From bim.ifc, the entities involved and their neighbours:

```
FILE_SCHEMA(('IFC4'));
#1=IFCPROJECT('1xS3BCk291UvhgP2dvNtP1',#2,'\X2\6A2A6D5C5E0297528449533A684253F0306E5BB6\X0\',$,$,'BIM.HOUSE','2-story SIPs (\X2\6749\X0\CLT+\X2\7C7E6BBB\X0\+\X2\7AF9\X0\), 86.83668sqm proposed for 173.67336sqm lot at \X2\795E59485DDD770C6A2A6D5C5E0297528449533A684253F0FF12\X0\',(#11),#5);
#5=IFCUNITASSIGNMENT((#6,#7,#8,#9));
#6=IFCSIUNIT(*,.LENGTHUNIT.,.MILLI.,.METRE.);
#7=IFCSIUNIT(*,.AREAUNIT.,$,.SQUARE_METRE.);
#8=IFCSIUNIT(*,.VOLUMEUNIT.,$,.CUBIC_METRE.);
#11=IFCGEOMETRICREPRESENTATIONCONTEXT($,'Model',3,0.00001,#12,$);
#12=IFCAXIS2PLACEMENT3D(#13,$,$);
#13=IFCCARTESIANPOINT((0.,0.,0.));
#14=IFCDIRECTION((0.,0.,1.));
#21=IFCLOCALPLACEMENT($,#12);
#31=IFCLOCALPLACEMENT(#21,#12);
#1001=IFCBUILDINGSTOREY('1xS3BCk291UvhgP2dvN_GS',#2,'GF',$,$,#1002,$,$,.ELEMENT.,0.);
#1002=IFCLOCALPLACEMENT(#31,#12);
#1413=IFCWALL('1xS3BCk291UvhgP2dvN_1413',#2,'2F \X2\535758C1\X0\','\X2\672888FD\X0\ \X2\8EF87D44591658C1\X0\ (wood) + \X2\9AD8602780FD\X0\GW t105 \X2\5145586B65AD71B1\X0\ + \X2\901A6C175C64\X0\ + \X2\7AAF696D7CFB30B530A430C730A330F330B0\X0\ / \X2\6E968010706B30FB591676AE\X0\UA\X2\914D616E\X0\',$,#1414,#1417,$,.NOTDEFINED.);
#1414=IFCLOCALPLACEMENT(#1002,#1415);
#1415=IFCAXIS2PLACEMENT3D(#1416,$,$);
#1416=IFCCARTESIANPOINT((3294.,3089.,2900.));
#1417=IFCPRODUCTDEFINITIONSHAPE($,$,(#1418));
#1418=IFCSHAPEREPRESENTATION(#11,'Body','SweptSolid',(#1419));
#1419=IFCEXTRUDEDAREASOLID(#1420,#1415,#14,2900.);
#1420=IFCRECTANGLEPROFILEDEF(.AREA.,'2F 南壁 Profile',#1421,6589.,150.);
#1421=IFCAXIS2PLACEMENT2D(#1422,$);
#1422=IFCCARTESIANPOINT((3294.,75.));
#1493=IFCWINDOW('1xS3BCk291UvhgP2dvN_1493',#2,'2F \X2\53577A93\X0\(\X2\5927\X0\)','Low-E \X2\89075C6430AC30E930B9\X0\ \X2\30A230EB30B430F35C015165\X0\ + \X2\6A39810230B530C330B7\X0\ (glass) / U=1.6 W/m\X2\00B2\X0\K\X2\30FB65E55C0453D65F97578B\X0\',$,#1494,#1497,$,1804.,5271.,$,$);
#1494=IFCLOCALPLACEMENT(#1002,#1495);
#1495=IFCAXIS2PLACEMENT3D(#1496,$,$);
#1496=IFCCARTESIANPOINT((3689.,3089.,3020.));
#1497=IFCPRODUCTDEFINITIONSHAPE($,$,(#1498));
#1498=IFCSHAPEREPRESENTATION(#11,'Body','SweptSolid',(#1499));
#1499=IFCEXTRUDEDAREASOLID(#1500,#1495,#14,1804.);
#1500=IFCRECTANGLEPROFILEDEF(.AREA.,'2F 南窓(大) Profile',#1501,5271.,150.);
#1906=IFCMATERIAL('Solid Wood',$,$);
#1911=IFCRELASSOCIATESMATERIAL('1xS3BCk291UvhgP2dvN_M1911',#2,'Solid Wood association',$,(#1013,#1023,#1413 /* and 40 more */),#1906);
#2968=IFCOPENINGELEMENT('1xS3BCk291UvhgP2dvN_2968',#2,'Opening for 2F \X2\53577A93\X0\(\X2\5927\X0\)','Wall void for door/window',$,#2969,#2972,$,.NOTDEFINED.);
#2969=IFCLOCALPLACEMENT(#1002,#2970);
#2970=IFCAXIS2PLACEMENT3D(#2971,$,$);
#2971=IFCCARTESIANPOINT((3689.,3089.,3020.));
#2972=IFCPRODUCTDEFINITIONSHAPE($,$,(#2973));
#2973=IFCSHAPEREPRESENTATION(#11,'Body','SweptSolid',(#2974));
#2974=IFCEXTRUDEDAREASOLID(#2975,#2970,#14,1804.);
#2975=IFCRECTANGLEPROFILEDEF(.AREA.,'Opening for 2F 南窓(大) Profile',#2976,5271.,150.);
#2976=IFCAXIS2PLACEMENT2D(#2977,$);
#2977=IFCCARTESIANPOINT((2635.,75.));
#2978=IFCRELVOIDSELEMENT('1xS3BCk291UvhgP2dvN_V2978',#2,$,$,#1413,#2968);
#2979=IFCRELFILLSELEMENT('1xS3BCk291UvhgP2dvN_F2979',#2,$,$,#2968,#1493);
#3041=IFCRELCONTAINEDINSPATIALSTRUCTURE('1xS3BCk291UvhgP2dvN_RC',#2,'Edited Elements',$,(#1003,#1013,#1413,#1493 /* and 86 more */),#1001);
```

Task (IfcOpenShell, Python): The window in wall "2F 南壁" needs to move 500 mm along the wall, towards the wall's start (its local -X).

```python
import ifcopenshell
import ifcopenshell.api.geometry
import ifcopenshell.util.placement
import ifcopenshell.util.unit

model = ifcopenshell.open("bim.ifc")
unit_scale = ifcopenshell.util.unit.calculate_unit_scale(model)

window = model.by_guid("1xS3BCk291UvhgP2dvN_1493")
opening = window.FillsVoids[0].RelatingOpeningElement
wall = opening.VoidsElements[0].RelatingBuildingElement

wall_matrix = ifcopenshell.util.placement.get_local_placement(wall.ObjectPlacement)
shift = wall_matrix[:3, 0] * -0.5 / unit_scale
before = ifcopenshell.util.placement.get_local_placement(window.ObjectPlacement)[:3, 3].copy()

# The window is not placed relative to its opening, so move both.
for product in (opening, window):
    matrix = ifcopenshell.util.placement.get_local_placement(product.ObjectPlacement)
    matrix[:3, 3] += shift
    ifcopenshell.api.geometry.edit_object_placement(model, product=product, matrix=matrix, is_si=False)

after = ifcopenshell.util.placement.get_local_placement(window.ObjectPlacement)[:3, 3]
print("window moved by", (after - before).round(3) + 0.0)

model.write("bim-out.ifc")
```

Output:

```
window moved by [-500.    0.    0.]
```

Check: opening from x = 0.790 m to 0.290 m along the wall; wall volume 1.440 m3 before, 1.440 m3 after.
